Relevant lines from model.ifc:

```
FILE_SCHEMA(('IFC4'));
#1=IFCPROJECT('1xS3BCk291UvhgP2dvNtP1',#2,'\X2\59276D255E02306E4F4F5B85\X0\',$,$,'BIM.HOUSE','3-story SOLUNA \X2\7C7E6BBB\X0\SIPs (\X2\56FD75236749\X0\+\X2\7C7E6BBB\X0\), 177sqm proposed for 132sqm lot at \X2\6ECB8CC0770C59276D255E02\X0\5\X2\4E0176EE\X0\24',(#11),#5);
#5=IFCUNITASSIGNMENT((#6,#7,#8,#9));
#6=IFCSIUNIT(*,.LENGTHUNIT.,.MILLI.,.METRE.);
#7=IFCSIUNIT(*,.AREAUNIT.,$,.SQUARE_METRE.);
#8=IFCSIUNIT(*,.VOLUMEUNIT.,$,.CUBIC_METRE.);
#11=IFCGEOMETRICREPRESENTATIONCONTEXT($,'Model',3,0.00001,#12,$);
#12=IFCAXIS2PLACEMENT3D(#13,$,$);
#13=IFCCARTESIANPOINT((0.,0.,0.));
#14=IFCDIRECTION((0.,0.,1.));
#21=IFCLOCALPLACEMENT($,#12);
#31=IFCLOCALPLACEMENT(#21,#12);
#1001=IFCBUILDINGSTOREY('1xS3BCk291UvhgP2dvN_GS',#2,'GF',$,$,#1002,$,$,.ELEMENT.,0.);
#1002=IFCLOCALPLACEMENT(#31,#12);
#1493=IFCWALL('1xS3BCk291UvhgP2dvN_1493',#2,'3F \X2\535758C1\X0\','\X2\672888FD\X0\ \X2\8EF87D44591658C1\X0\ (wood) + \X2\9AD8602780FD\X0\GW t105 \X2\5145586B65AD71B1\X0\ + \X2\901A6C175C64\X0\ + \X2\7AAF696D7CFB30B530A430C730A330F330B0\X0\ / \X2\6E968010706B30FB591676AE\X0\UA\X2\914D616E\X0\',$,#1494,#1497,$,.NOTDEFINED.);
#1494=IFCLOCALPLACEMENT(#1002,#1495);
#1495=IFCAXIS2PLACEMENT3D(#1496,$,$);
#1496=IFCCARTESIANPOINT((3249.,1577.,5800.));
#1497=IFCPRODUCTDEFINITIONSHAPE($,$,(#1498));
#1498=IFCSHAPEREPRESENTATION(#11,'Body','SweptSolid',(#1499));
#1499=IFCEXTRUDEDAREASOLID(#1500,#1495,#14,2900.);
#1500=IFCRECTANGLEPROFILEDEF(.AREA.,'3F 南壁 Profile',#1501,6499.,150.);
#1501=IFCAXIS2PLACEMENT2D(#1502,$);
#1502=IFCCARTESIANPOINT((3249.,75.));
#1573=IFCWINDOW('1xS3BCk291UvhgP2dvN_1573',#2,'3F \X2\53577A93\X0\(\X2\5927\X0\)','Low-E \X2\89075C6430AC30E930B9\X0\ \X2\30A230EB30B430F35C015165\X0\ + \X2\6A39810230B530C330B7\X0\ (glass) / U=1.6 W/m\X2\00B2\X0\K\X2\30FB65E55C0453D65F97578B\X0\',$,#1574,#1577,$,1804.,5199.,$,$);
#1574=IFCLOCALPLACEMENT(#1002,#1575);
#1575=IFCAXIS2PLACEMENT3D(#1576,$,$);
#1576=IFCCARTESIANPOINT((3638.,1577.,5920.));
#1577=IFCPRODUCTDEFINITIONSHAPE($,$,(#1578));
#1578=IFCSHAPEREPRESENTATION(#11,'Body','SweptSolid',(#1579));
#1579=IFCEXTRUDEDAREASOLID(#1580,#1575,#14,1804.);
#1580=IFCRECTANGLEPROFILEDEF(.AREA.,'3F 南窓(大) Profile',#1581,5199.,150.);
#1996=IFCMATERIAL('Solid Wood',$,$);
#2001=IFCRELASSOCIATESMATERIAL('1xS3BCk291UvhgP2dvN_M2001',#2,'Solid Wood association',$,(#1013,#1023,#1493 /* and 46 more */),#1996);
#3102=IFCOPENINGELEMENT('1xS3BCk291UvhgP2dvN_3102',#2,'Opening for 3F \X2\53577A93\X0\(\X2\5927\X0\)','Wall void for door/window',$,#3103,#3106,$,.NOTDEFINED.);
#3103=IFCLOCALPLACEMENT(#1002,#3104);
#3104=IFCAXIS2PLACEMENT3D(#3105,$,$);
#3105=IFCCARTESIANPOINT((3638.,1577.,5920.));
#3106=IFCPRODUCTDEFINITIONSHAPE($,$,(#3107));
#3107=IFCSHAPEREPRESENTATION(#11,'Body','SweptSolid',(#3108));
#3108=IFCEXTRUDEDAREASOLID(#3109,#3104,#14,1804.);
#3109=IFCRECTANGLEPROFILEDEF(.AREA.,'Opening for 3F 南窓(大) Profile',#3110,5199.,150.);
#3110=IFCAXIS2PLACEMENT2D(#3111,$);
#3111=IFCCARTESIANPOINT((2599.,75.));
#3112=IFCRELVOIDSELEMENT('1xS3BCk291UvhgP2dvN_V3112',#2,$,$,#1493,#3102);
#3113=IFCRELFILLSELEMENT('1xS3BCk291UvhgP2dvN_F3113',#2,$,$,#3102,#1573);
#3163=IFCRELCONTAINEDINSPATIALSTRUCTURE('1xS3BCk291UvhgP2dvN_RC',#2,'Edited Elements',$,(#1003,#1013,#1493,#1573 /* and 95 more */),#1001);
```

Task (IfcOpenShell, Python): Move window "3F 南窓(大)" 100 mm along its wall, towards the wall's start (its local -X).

```python
import ifcopenshell
import ifcopenshell.api.geometry
import ifcopenshell.util.placement
import ifcopenshell.util.unit

model = ifcopenshell.open("model.ifc")
unit_scale = ifcopenshell.util.unit.calculate_unit_scale(model)

window = model.by_guid("1xS3BCk291UvhgP2dvN_1573")
opening = window.FillsVoids[0].RelatingOpeningElement
wall = opening.VoidsElements[0].RelatingBuildingElement

wall_matrix = ifcopenshell.util.placement.get_local_placement(wall.ObjectPlacement)
shift = wall_matrix[:3, 0] * -0.1 / unit_scale
before = ifcopenshell.util.placement.get_local_placement(window.ObjectPlacement)[:3, 3].copy()

# The window is not placed relative to its opening, so move both.
for product in (opening, window):
    matrix = ifcopenshell.util.placement.get_local_placement(product.ObjectPlacement)
    matrix[:3, 3] += shift
    ifcopenshell.api.geometry.edit_object_placement(model, product=product, matrix=matrix, is_si=False)

after = ifcopenshell.util.placement.get_local_placement(window.ObjectPlacement)[:3, 3]
print("window moved by", (after - before).round(3) + 0.0)

model.write("model_edited.ifc")
```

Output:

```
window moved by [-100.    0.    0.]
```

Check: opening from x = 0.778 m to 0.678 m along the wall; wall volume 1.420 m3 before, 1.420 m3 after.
